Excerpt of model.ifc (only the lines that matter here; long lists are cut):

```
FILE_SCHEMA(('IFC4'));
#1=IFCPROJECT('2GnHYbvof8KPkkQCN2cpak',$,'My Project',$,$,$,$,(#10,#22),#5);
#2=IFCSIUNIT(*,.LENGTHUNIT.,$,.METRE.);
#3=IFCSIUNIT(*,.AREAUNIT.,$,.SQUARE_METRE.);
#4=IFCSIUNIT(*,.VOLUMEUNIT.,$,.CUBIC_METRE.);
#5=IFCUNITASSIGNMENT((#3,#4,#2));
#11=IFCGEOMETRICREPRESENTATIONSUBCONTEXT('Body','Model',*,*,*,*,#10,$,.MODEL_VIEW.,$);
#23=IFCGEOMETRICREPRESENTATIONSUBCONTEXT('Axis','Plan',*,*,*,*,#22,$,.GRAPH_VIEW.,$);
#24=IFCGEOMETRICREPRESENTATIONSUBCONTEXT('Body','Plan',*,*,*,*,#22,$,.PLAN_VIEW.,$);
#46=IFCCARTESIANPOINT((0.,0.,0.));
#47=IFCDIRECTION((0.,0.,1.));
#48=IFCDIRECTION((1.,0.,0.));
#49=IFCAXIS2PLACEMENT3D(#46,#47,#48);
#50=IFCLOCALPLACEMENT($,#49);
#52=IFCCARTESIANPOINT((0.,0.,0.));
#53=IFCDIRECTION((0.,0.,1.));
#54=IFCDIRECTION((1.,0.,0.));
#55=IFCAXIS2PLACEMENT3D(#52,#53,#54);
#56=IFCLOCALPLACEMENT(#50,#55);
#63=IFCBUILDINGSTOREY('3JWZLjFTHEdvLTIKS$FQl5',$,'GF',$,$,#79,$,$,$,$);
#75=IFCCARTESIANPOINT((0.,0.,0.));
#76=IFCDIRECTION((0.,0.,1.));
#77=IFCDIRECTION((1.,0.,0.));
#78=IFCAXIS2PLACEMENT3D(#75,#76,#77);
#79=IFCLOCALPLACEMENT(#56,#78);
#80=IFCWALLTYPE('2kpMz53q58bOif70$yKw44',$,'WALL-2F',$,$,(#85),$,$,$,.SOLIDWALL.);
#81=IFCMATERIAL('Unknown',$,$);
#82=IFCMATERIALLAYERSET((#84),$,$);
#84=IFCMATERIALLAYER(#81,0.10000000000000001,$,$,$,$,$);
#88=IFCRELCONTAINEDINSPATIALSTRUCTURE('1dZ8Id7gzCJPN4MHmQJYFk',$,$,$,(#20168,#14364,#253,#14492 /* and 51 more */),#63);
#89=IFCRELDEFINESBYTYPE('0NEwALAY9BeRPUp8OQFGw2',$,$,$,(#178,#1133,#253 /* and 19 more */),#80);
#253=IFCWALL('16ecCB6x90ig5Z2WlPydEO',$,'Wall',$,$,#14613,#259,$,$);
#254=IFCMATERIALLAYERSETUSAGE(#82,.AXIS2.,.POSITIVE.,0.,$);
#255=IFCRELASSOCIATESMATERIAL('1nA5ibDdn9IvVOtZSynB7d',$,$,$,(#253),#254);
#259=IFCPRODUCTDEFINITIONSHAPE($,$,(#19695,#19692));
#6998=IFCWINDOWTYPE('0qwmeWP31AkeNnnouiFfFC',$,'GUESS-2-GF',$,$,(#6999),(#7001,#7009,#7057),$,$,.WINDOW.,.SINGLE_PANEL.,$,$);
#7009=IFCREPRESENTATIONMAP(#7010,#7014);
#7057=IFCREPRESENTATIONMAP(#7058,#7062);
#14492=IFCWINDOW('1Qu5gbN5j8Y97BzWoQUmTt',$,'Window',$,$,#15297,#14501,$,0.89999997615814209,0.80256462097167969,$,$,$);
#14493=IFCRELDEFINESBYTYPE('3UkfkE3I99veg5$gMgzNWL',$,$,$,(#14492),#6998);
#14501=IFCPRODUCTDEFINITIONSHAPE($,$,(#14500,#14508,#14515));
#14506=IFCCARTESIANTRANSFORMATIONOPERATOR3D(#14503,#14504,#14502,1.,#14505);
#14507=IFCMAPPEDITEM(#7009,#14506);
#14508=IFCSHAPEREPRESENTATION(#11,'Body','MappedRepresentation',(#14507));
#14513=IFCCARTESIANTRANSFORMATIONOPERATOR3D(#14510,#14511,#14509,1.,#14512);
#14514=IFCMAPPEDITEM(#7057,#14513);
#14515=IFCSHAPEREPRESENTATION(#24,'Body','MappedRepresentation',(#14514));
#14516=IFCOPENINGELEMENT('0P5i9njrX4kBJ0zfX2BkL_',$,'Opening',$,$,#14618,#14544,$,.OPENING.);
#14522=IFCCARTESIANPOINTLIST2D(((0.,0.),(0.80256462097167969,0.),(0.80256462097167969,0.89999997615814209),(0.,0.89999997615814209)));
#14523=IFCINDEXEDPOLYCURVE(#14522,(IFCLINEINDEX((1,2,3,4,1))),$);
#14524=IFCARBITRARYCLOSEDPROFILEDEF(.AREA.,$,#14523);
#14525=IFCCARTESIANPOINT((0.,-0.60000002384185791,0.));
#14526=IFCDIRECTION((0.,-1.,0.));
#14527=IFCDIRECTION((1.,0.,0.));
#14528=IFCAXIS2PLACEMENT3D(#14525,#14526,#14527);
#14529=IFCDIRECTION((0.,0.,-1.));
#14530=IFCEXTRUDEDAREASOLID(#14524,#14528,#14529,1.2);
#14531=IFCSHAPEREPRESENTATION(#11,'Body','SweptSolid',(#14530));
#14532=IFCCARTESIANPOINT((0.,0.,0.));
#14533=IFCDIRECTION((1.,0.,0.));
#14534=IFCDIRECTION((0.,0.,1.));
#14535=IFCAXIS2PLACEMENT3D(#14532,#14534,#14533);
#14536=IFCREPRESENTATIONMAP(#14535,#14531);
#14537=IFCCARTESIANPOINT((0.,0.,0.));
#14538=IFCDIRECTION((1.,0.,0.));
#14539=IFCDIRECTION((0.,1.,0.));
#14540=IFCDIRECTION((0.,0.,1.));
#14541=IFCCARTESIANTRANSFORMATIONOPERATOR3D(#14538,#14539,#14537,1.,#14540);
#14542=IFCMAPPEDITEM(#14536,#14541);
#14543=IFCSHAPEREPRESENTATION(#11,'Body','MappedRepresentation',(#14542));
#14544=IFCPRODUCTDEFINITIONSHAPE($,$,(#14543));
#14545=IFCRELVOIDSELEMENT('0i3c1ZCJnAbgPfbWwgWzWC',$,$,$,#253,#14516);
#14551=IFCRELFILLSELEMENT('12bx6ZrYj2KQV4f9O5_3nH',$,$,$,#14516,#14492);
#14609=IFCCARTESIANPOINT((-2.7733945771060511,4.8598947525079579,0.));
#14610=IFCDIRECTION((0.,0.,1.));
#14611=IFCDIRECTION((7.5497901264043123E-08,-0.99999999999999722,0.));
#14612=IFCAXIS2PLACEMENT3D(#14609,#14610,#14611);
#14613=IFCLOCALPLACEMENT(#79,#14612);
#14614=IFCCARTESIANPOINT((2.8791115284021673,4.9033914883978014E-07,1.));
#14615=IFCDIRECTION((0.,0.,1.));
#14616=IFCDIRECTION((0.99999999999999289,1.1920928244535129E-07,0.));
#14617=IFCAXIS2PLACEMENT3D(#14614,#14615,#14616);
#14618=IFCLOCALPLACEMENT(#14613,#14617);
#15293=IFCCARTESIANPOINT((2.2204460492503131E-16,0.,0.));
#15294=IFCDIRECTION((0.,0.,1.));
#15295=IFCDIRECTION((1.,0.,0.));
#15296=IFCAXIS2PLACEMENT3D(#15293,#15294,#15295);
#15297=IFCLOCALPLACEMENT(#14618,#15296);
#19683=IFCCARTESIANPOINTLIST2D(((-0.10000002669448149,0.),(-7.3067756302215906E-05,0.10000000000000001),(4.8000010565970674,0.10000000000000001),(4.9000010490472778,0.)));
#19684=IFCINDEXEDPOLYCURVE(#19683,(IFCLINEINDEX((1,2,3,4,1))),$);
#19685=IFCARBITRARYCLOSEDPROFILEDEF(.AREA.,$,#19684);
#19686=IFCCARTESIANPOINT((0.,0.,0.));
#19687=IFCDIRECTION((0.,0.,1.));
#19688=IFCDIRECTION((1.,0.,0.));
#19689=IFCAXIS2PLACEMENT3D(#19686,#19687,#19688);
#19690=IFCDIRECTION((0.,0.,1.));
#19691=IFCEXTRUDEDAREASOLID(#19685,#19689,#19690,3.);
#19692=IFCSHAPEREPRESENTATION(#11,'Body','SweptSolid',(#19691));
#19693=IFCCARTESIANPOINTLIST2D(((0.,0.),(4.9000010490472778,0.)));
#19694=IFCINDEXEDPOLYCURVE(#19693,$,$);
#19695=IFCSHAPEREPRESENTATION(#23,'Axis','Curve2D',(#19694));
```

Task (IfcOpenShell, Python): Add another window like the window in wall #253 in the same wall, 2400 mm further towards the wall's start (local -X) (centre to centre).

```python
import ifcopenshell
import ifcopenshell.api.feature
import ifcopenshell.api.geometry
import ifcopenshell.api.root
import ifcopenshell.geom
import ifcopenshell.util.element
import ifcopenshell.util.placement
import ifcopenshell.util.shape

model = ifcopenshell.open("model.ifc")
settings = ifcopenshell.geom.settings()


def volume(element):
    """Net volume in cubic metres, openings subtracted."""
    shape = ifcopenshell.geom.create_shape(settings, element)
    return ifcopenshell.util.shape.get_volume(shape.geometry)


window = model.by_guid("1Qu5gbN5j8Y97BzWoQUmTt")
opening = window.FillsVoids[0].RelatingOpeningElement
wall = opening.VoidsElements[0].RelatingBuildingElement
before = volume(wall)
shift = ifcopenshell.util.placement.get_local_placement(wall.ObjectPlacement)[:3, 0] * -2.4

# copy_class copies the void relationship, type, container and properties, but no geometry.
new_opening = ifcopenshell.api.root.copy_class(model, product=opening)
new_opening.Representation = ifcopenshell.util.element.copy_deep(
    model, opening.Representation, exclude=["IfcGeometricRepresentationContext", "IfcRepresentationMap"]
)
new_window = ifcopenshell.api.root.copy_class(model, product=window)
new_window.Representation = ifcopenshell.util.element.copy_deep(
    model, window.Representation, exclude=["IfcGeometricRepresentationContext", "IfcRepresentationMap"]
)
ifcopenshell.api.feature.add_filling(model, opening=new_opening, element=new_window)

for old, new in ((opening, new_opening), (window, new_window)):
    matrix = ifcopenshell.util.placement.get_local_placement(old.ObjectPlacement)
    matrix[:3, 3] += shift
    ifcopenshell.api.geometry.edit_object_placement(model, product=new, matrix=matrix, is_si=False)

after = volume(wall)

print(f"wall volume {before:.3f} -> {after:.3f} m3")

model.write("model_v2.ifc")
```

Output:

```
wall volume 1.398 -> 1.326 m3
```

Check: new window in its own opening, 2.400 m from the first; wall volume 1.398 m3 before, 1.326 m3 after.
